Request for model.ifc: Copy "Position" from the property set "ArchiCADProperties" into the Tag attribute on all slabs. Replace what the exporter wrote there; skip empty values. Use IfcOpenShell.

First a look at what the model holds.

```python
import ifcopenshell
import ifcopenshell.util.element

model = ifcopenshell.open("model.ifc")
print(model.schema)
slabs = model.by_type("IfcSlab")
print(len(slabs), "slabs")
for e in slabs[:8]:
    source = ifcopenshell.util.element.get_pset(e, "ArchiCADProperties", "Position")
    target = e.Tag
    print(e.id(), repr(source), repr(target), sep=" | ")
```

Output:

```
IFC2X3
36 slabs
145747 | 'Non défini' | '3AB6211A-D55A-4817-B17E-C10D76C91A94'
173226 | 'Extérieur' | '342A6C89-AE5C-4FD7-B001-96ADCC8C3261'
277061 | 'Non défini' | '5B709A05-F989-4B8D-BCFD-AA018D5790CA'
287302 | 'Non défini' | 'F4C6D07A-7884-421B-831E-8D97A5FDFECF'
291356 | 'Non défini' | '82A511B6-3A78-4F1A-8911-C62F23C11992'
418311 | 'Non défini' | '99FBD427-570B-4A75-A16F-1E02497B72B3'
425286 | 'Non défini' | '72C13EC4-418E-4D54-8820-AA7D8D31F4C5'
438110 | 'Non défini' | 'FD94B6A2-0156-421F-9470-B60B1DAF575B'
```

```python
import ifcopenshell
import ifcopenshell.util.element

model = ifcopenshell.open("model.ifc")

count = 0
for e in model.by_type("IfcSlab"):
    value = ifcopenshell.util.element.get_pset(e, "ArchiCADProperties", "Position")
    current = e.Tag
    if not value or not value.strip() or current == value:
        continue
    e.Tag = value
    count += 1

print(count, "slabs updated")

model.write("model-out.ifc")
```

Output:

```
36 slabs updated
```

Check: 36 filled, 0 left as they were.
